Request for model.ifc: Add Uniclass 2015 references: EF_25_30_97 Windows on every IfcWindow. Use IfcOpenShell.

First a look at what the model holds.

```python
import ifcopenshell

model = ifcopenshell.open("model.ifc")
print(model.schema)
print("classifications:", [c.Name for c in model.by_type("IfcClassification")])
for ifc_class in ("IfcDoor", "IfcRoof", "IfcStair", "IfcWall", "IfcWindow"):
    print(ifc_class, len(model.by_type(ifc_class)))
```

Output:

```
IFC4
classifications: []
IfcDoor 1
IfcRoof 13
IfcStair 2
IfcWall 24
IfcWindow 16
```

```python
import ifcopenshell
import ifcopenshell.api.classification

model = ifcopenshell.open("model.ifc")

system = ifcopenshell.api.classification.add_classification(model, classification="Uniclass 2015")

codes = {
    "IfcWindow": ("EF_25_30_97", "Windows"),
}
for ifc_class, (code, name) in codes.items():
    products = model.by_type(ifc_class)
    ifcopenshell.api.classification.add_reference(
        model, products=products, classification=system, identification=code, name=name
    )
    print(code, len(products))

model.write("model-out.ifc")
```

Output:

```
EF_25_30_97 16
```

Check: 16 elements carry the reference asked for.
